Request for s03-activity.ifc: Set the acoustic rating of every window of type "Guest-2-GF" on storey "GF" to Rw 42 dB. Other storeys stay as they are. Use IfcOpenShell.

First a look at what the model holds.

```python
import ifcopenshell
import ifcopenshell.util.element

model = ifcopenshell.open("s03-activity.ifc")
print(model.schema)
storey = next(s for s in model.by_type("IfcBuildingStorey") if s.Name == "GF")
windows = [e for e in ifcopenshell.util.element.get_decomposition(storey) if e.is_a("IfcWindow")]
seen = {}
for e in windows:
    element_type = ifcopenshell.util.element.get_type(e)
    key = (element_type.Name if element_type != e and element_type else None, ifcopenshell.util.element.get_pset(e, "Pset_WindowCommon", "AcousticRating"))
    seen[key] = seen.get(key, 0) + 1
for (name, value), count in sorted(seen.items(), key=str):
    print(count, "x", name, "|", value)
```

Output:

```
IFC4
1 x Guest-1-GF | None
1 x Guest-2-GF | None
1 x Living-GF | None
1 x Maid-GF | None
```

```python
import ifcopenshell
import ifcopenshell.api.pset
import ifcopenshell.util.element

model = ifcopenshell.open("s03-activity.ifc")

storey = next(s for s in model.by_type("IfcBuildingStorey") if s.Name == "GF")
windows = [e for e in ifcopenshell.util.element.get_decomposition(storey) if e.is_a("IfcWindow")]

count = 0
for e in windows:
    element_type = ifcopenshell.util.element.get_type(e)
    if element_type in (None, e) or element_type.Name != "Guest-2-GF":
        continue
    # add_pset returns the element's existing set when there is one.
    pset = ifcopenshell.api.pset.add_pset(model, product=e, name="Pset_WindowCommon")
    ifcopenshell.api.pset.edit_pset(model, pset=pset, properties={"AcousticRating": "Rw 42 dB"})
    count += 1

print(count, "windows updated")

model.write("s03-activity-out.ifc")
```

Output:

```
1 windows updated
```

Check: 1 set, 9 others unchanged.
